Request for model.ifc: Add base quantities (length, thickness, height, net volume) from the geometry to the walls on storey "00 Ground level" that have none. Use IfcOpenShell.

First a look at what the model holds.

```python
import ifcopenshell
import ifcopenshell.util.element
import ifcopenshell.util.unit

model = ifcopenshell.open("model.ifc")
print(model.schema)
for unit_type in ("LENGTHUNIT", "AREAUNIT", "VOLUMEUNIT"):
    print(unit_type, ifcopenshell.util.unit.calculate_unit_scale(model, unit_type))
storey = next(s for s in model.by_type("IfcBuildingStorey") if s.Name == "00 Ground level")
walls = [e for e in ifcopenshell.util.element.get_decomposition(storey) if e.is_a("IfcWall")]
for e in sorted(walls, key=lambda e: e.id()):
    print(e.id(), e.is_a(), e.Name, list(ifcopenshell.util.element.get_psets(e, qtos_only=True)), sep=" | ")
```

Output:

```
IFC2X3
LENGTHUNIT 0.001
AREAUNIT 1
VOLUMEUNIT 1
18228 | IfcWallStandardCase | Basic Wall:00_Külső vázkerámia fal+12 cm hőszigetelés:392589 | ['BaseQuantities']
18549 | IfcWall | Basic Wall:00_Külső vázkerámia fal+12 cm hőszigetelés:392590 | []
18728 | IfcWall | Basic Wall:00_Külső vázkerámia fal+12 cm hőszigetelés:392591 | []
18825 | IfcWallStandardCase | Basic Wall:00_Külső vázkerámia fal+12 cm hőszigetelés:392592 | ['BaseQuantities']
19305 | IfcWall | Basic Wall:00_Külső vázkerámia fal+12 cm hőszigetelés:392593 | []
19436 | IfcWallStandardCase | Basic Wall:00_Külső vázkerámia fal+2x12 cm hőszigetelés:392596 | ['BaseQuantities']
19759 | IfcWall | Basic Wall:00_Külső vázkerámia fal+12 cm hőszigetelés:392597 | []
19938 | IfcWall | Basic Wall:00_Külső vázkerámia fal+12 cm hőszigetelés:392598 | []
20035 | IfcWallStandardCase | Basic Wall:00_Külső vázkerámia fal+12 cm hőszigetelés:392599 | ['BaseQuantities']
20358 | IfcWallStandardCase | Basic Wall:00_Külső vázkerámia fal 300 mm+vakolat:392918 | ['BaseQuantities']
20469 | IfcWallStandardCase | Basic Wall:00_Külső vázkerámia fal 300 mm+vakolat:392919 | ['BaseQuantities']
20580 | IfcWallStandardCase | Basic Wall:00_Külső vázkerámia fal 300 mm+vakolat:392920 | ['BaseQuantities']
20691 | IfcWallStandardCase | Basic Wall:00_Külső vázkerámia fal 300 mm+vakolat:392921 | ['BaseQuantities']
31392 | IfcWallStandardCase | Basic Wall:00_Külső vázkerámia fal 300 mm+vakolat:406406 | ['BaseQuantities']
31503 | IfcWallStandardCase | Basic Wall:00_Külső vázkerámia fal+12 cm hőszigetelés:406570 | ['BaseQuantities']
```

```python
import ifcopenshell
import ifcopenshell.api.pset
import ifcopenshell.geom
import ifcopenshell.util.element
import ifcopenshell.util.shape
import ifcopenshell.util.unit

model = ifcopenshell.open("model.ifc")
unit_scale = ifcopenshell.util.unit.calculate_unit_scale(model)
volume_scale = ifcopenshell.util.unit.calculate_unit_scale(model, "VOLUMEUNIT")
settings = ifcopenshell.geom.settings()

storey = next(s for s in model.by_type("IfcBuildingStorey") if s.Name == "00 Ground level")
walls = [e for e in ifcopenshell.util.element.get_decomposition(storey) if e.is_a("IfcWall")]

for e in sorted(walls, key=lambda e: e.id()):
    if ifcopenshell.util.element.get_psets(e, qtos_only=True, should_inherit=False):
        continue
    # Geometry comes back in metres, in the element's own axes.
    shape = ifcopenshell.geom.create_shape(settings, e)
    values = {
        "Length": ifcopenshell.util.shape.get_x(shape.geometry) / unit_scale,
        "Width": ifcopenshell.util.shape.get_y(shape.geometry) / unit_scale,
        "Height": ifcopenshell.util.shape.get_z(shape.geometry) / unit_scale,
        "NetVolume": ifcopenshell.util.shape.get_volume(shape.geometry) / volume_scale,
    }
    qto = ifcopenshell.api.pset.add_qto(model, product=e, name="BaseQuantities")
    ifcopenshell.api.pset.edit_qto(model, qto=qto, properties=values)
    print(e.id(), {k: round(v, 3) for k, v in values.items()})

model.write("model-out.ifc")
```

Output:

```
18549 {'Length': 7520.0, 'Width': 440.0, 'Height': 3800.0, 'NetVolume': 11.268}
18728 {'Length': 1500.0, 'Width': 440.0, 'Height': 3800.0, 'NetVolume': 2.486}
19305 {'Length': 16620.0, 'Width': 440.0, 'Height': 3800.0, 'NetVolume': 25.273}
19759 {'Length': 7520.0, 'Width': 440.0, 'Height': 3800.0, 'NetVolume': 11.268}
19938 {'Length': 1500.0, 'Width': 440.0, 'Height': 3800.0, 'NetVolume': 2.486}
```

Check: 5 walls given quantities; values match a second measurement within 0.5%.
